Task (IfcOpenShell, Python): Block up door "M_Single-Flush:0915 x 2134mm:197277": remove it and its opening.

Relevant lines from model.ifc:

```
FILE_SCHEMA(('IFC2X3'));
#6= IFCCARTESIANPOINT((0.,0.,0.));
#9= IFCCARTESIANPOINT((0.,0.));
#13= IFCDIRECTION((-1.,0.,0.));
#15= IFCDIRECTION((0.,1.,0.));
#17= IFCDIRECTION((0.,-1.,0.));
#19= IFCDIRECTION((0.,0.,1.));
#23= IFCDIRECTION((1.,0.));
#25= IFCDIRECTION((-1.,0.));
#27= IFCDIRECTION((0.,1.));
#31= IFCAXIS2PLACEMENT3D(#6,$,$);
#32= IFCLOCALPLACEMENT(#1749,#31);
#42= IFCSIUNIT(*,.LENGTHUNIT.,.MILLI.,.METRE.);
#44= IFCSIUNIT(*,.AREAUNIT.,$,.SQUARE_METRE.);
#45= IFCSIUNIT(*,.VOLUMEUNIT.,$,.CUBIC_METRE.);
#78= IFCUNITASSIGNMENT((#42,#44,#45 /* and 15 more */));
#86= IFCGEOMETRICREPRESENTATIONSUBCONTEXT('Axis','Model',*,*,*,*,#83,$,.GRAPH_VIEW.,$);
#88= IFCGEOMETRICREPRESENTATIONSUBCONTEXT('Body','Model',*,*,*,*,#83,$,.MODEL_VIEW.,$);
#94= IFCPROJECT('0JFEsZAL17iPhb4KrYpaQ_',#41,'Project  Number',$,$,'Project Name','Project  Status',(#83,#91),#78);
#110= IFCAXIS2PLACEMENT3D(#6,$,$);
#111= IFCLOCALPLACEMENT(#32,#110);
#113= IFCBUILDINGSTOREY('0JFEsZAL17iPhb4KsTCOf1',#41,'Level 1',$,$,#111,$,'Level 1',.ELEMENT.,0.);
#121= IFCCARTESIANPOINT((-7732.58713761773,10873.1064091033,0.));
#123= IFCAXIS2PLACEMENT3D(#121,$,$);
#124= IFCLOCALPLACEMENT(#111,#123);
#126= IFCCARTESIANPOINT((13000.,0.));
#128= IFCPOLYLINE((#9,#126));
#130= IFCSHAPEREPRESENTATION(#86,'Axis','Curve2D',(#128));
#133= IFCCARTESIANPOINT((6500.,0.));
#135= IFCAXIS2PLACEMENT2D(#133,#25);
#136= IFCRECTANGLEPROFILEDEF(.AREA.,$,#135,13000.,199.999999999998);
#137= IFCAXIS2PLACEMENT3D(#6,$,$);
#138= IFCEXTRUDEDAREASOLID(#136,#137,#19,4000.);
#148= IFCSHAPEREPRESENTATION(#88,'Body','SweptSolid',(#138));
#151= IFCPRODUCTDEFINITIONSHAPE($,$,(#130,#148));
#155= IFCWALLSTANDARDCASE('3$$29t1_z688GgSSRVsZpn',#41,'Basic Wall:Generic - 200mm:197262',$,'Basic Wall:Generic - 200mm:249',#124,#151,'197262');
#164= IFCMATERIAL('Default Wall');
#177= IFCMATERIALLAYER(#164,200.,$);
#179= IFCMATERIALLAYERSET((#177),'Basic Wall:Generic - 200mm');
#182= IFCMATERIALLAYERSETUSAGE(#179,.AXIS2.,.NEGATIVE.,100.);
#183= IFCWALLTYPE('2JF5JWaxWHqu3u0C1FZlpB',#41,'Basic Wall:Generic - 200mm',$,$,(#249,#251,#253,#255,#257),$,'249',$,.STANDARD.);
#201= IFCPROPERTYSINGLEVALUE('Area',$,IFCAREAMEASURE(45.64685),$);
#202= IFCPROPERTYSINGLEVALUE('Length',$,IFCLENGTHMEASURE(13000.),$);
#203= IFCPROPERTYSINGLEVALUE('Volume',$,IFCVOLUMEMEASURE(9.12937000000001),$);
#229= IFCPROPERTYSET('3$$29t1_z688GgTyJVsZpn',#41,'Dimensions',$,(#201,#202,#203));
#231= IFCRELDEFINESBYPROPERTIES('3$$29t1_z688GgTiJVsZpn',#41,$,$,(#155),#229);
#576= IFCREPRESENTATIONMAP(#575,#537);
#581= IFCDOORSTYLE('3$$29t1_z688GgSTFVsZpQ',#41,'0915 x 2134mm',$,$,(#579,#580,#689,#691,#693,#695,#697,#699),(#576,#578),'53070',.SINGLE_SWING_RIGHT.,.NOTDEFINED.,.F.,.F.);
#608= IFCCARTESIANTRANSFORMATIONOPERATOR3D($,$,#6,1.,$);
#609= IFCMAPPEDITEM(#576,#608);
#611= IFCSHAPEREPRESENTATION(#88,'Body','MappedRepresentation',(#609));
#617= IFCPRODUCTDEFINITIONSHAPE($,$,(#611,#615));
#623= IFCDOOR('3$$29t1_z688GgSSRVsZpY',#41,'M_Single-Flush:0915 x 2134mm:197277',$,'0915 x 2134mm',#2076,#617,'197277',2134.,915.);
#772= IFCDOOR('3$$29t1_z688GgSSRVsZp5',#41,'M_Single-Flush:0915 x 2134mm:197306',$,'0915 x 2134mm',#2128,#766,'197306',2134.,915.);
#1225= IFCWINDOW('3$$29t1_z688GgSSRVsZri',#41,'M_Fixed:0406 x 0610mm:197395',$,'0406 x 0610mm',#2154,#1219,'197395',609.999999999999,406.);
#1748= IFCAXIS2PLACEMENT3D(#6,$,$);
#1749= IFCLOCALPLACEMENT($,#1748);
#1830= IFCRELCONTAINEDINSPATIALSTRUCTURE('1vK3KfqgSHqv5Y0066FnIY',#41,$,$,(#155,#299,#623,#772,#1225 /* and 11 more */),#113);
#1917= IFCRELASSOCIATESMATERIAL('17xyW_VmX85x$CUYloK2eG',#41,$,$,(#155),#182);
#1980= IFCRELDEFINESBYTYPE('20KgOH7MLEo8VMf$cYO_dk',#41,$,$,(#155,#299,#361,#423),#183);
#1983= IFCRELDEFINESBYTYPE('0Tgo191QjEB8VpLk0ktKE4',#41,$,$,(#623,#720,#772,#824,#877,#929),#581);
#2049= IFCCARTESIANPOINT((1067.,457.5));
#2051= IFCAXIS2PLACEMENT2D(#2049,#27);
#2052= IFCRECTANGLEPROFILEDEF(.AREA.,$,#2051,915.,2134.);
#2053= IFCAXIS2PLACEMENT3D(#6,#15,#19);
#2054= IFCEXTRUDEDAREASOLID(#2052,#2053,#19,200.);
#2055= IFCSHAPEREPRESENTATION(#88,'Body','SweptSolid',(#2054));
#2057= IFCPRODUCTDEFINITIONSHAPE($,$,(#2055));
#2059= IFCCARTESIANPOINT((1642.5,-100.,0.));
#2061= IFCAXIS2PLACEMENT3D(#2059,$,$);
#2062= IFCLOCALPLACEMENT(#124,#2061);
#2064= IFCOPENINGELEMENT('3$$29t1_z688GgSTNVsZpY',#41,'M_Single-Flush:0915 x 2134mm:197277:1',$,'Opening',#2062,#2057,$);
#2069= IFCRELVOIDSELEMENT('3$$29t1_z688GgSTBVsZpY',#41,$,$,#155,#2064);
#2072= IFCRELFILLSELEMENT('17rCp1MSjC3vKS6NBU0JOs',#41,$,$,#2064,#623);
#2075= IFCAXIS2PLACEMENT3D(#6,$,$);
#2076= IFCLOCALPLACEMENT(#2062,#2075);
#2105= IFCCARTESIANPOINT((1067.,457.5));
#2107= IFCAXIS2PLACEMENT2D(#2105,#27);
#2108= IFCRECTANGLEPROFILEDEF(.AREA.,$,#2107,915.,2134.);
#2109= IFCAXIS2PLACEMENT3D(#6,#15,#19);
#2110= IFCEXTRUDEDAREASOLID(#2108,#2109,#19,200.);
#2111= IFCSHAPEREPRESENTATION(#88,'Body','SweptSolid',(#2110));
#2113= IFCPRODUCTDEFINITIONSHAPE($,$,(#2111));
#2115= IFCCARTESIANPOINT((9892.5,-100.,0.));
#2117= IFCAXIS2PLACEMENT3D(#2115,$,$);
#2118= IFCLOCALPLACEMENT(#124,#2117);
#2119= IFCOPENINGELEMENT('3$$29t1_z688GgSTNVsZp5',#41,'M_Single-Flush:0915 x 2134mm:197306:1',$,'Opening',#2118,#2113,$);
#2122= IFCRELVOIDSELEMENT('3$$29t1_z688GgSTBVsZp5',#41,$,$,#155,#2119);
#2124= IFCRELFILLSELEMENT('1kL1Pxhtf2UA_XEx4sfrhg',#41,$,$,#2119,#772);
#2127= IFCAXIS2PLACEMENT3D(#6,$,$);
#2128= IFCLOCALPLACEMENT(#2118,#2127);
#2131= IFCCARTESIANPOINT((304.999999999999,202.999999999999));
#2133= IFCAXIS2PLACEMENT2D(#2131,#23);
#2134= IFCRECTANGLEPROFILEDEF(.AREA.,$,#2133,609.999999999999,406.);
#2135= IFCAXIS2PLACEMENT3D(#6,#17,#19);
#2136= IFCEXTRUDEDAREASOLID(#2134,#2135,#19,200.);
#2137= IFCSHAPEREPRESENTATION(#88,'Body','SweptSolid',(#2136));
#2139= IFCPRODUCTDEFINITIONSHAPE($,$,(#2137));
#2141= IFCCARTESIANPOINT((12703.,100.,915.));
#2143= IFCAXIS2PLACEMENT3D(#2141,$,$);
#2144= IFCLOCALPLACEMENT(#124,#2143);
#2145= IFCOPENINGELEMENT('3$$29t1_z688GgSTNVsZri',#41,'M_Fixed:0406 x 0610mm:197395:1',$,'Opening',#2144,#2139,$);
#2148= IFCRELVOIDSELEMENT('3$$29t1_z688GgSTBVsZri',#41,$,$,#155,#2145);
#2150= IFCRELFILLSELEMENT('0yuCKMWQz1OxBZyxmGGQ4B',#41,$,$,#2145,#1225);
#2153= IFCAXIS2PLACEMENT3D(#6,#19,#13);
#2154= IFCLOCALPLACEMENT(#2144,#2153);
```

```python
import ifcopenshell
import ifcopenshell.api.feature
import ifcopenshell.api.pset
import ifcopenshell.api.root
import ifcopenshell.geom
import ifcopenshell.util.element
import ifcopenshell.util.shape
import ifcopenshell.util.unit

model = ifcopenshell.open("model.ifc")
area_scale = ifcopenshell.util.unit.calculate_unit_scale(model, "AREAUNIT")
volume_scale = ifcopenshell.util.unit.calculate_unit_scale(model, "VOLUMEUNIT")
settings = ifcopenshell.geom.settings()


def volume(element):
    """Net volume in cubic metres, openings subtracted."""
    shape = ifcopenshell.geom.create_shape(settings, element)
    return ifcopenshell.util.shape.get_volume(shape.geometry)


door = model.by_id(623)
opening = door.FillsVoids[0].RelatingOpeningElement
wall = opening.VoidsElements[0].RelatingBuildingElement
before = volume(wall)

ifcopenshell.api.root.remove_product(model, product=door)
ifcopenshell.api.feature.remove_feature(model, feature=opening)

after = volume(wall)
thickness = 0.2  # wall thickness in metres

# Update the wall's stored quantities.
pset = model.by_id(ifcopenshell.util.element.get_pset(wall, "Dimensions", should_inherit=False)["id"])
ifcopenshell.api.pset.edit_pset(model, pset=pset, properties={
    "Area": model.create_entity("IfcAreaMeasure", after / thickness / area_scale),
    "Volume": model.create_entity("IfcVolumeMeasure", after / volume_scale),
})

print(f"wall volume {before:.3f} -> {after:.3f} m3")

model.write("model_updated.ifc")
```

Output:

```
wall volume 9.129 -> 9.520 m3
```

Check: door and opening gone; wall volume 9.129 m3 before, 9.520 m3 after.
